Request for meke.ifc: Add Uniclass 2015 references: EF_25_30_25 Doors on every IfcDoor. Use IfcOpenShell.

First a look at what the model holds.

```python
import ifcopenshell

model = ifcopenshell.open("meke.ifc")
print(model.schema)
print("classifications:", [c.Name for c in model.by_type("IfcClassification")])
for ifc_class in ("IfcDoor", "IfcRoof", "IfcStair", "IfcWall", "IfcWindow"):
    print(ifc_class, len(model.by_type(ifc_class)))
```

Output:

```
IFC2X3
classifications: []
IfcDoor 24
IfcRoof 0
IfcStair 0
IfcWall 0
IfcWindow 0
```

```python
import ifcopenshell
import ifcopenshell.api.classification

model = ifcopenshell.open("meke.ifc")

# IFC2X3 requires Source and Edition and has no link from the project to the system.
system = model.create_entity("IfcClassification", Source="NBS", Edition="2015", Name="Uniclass 2015")

codes = {
    "IfcDoor": ("EF_25_30_25", "Doors"),
}
for ifc_class, (code, name) in codes.items():
    products = model.by_type(ifc_class)
    ifcopenshell.api.classification.add_reference(
        model, products=products, classification=system, identification=code, name=name
    )
    print(code, len(products))

model.write("meke_v2.ifc")
```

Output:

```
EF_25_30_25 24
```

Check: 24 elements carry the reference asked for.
